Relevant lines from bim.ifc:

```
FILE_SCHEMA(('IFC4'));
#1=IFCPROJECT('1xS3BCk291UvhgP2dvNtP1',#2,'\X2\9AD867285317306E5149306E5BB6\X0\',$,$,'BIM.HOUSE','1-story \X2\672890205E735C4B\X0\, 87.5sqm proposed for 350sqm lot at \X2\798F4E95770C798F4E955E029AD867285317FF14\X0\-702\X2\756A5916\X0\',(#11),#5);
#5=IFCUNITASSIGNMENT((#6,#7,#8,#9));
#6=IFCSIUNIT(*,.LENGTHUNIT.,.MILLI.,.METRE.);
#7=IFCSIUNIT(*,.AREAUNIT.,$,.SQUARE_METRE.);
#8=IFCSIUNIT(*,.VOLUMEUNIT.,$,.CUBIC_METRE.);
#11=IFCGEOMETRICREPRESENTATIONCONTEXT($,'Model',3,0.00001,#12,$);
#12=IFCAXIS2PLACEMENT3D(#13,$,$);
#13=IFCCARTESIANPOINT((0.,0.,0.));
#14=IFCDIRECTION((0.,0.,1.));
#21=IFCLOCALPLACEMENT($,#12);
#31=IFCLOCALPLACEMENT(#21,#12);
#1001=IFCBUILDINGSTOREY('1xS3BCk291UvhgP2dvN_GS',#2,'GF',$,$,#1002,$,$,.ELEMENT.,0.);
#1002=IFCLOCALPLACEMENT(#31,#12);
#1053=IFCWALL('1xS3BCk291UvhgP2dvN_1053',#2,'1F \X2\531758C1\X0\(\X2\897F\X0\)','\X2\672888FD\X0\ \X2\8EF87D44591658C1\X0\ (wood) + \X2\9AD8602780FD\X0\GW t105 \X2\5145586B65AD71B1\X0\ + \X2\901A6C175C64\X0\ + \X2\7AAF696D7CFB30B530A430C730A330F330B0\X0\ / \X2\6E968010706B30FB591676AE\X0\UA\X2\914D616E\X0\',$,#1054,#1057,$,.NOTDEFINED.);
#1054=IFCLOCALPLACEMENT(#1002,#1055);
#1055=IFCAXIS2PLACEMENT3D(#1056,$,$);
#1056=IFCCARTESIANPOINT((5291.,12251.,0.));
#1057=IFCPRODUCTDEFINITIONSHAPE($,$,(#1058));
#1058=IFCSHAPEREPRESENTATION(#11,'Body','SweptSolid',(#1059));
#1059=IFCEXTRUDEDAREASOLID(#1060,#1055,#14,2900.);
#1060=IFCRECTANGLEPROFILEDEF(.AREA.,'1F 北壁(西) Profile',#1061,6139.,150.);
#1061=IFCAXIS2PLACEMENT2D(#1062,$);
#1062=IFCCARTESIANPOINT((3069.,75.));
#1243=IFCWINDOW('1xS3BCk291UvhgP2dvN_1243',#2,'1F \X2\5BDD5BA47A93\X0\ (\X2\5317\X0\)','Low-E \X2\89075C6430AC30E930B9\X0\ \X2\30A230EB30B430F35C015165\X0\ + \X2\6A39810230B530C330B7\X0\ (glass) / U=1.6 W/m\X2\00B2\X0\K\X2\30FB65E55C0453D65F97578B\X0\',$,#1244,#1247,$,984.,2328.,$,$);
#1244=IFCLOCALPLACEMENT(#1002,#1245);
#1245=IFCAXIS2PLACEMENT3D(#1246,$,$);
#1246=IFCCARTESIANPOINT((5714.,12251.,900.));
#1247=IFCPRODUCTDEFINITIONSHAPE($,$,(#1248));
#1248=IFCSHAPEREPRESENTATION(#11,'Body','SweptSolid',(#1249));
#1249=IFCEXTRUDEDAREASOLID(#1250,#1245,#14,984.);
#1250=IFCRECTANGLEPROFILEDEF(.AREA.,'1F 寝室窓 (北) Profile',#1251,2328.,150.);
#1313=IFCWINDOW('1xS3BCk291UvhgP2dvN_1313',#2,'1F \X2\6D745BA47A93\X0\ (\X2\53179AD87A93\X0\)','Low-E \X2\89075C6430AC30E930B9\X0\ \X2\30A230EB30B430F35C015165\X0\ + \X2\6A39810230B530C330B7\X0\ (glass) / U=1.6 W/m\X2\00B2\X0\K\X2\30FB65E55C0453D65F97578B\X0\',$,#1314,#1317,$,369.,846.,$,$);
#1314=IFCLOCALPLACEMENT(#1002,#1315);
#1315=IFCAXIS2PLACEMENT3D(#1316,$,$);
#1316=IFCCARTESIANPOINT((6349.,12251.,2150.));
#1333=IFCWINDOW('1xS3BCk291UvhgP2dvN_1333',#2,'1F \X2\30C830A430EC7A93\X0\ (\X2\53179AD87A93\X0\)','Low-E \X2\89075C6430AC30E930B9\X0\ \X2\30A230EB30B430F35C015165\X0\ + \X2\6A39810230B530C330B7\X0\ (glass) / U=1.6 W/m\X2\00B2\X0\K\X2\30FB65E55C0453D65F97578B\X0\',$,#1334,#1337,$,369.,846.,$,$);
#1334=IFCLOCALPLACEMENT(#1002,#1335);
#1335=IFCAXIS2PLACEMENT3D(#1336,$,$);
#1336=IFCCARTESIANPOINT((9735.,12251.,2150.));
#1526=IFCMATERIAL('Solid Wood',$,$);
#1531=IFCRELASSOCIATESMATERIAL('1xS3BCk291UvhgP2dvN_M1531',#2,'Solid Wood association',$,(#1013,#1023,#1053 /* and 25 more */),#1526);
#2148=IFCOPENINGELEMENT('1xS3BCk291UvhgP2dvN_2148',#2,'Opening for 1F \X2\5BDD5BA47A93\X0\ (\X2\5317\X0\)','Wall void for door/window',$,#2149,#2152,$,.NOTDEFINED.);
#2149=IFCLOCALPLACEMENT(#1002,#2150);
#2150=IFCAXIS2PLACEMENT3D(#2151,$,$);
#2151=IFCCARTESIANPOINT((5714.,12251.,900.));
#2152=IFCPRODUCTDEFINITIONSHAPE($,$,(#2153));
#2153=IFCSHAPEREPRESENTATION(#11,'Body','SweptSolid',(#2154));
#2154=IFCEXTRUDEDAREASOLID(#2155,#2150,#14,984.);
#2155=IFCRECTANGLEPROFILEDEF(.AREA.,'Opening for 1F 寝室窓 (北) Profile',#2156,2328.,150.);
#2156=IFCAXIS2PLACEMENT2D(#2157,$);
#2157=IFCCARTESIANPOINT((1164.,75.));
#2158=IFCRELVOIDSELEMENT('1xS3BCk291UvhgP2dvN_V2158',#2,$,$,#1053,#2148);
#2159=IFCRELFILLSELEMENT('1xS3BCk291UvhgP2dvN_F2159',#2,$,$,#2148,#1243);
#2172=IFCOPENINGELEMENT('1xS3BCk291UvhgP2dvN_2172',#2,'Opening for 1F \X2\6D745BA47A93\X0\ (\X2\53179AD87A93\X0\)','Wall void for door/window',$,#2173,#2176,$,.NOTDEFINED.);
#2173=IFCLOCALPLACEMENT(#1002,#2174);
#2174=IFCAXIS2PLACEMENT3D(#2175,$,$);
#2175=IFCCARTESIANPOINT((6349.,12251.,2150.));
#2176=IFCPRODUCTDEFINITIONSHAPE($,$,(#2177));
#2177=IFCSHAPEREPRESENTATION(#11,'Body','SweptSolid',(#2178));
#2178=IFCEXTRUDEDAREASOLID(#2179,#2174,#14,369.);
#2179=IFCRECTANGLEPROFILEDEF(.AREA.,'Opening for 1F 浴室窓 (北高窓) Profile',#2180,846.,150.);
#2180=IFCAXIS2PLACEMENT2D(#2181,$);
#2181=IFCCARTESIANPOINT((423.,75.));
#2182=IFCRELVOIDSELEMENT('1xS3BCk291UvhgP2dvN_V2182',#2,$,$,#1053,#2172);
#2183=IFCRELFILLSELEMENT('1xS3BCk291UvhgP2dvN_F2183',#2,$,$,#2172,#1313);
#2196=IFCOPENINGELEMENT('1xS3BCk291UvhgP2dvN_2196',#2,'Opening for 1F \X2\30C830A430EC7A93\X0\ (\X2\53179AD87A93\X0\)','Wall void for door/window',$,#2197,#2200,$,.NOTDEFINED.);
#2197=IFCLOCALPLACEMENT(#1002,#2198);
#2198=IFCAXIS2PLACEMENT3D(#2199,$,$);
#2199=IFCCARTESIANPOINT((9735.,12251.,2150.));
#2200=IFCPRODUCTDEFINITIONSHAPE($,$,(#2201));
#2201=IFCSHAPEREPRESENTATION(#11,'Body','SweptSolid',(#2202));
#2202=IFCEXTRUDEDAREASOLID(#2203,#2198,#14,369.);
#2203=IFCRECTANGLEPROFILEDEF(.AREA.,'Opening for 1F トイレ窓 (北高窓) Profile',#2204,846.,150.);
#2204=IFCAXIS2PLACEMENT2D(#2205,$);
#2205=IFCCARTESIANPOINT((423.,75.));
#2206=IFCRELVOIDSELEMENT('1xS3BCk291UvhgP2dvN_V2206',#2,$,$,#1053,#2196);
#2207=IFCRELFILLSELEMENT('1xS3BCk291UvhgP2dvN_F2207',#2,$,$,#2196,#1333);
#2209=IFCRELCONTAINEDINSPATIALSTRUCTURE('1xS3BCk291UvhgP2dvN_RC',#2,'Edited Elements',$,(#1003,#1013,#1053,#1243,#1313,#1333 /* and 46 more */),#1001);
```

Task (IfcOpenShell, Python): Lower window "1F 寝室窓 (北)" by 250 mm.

```python
import numpy as np
import ifcopenshell
import ifcopenshell.api.geometry
import ifcopenshell.util.placement
import ifcopenshell.util.unit

model = ifcopenshell.open("bim.ifc")
unit_scale = ifcopenshell.util.unit.calculate_unit_scale(model)

window = model.by_id(1243)
opening = window.FillsVoids[0].RelatingOpeningElement
dz = -250.0

shift = np.array([0.0, 0.0, dz])
# The window is not placed relative to its opening, so move both.
for product in (opening, window):
    matrix = ifcopenshell.util.placement.get_local_placement(product.ObjectPlacement)
    matrix[:3, 3] += shift
    ifcopenshell.api.geometry.edit_object_placement(model, product=product, matrix=matrix, is_si=False)

print(f"moved by {dz * unit_scale:+.3f} m")

model.write("bim_v2.ifc")
```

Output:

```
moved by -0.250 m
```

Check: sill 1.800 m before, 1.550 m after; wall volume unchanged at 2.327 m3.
